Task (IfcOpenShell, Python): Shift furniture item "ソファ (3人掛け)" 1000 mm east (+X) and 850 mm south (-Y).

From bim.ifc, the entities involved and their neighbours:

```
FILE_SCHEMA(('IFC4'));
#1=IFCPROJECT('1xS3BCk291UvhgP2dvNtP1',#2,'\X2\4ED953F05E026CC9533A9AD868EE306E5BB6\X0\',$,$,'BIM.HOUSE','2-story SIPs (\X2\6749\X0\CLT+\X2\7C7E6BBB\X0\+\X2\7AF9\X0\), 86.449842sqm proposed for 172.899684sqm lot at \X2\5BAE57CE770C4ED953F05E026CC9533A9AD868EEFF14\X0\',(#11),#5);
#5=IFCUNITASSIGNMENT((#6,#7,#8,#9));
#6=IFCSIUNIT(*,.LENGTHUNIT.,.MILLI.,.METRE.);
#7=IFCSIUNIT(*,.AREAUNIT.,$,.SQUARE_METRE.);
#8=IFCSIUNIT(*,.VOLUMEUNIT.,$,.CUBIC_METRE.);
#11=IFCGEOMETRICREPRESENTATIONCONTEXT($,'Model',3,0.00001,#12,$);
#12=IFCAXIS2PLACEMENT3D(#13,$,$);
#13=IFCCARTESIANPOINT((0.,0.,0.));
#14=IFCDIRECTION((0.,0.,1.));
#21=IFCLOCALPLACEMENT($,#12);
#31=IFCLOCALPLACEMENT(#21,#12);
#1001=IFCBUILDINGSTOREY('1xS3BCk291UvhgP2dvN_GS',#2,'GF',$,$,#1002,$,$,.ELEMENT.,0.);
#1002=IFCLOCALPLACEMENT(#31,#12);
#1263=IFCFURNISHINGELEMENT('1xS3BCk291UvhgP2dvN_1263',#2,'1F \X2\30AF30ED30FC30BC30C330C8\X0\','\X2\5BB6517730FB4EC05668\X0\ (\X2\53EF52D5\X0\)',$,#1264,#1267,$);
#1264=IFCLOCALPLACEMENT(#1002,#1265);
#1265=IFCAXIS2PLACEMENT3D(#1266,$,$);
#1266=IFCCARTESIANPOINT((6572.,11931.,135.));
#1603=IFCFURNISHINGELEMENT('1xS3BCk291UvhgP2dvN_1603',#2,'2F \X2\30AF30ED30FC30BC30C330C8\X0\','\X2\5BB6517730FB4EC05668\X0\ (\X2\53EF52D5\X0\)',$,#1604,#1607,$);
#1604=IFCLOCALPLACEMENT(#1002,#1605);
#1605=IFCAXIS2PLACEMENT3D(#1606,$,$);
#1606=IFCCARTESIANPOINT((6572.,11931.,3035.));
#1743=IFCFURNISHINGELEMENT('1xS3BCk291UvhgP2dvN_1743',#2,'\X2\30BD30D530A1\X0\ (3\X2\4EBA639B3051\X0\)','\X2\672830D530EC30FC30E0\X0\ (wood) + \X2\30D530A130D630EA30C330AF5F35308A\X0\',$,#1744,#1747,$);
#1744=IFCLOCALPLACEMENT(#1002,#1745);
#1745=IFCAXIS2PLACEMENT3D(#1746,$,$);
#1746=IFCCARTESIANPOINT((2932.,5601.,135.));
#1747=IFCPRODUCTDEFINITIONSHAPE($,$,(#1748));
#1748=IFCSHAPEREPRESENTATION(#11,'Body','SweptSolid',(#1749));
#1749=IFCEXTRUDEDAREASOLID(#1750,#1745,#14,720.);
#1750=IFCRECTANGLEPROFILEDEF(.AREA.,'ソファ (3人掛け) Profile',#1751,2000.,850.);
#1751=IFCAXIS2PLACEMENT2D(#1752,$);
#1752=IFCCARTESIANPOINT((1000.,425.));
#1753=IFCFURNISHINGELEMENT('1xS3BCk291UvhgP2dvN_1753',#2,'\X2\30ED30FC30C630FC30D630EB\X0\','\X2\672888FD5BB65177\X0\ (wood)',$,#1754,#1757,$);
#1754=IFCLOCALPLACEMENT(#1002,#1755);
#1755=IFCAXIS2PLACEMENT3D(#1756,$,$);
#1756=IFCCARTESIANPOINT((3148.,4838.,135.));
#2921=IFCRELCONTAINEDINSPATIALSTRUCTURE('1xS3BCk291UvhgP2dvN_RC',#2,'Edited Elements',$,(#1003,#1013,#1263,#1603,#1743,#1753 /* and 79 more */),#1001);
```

```python
import ifcopenshell
import ifcopenshell.api.geometry
import ifcopenshell.util.placement

model = ifcopenshell.open("bim.ifc")

item = model.by_guid("1xS3BCk291UvhgP2dvN_1743")
matrix = ifcopenshell.util.placement.get_local_placement(item.ObjectPlacement)
matrix[0, 3] += 1000.0
matrix[1, 3] -= 850.0
ifcopenshell.api.geometry.edit_object_placement(model, product=item, matrix=matrix, is_si=False)

print(ifcopenshell.util.placement.get_local_placement(item.ObjectPlacement).round(3) + 0.0)

model.write("bim-out.ifc")
```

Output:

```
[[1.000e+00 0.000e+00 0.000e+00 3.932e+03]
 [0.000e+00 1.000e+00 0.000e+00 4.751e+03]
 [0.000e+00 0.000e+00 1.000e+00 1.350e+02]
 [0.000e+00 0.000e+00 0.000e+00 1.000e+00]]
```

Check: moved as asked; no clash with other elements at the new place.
